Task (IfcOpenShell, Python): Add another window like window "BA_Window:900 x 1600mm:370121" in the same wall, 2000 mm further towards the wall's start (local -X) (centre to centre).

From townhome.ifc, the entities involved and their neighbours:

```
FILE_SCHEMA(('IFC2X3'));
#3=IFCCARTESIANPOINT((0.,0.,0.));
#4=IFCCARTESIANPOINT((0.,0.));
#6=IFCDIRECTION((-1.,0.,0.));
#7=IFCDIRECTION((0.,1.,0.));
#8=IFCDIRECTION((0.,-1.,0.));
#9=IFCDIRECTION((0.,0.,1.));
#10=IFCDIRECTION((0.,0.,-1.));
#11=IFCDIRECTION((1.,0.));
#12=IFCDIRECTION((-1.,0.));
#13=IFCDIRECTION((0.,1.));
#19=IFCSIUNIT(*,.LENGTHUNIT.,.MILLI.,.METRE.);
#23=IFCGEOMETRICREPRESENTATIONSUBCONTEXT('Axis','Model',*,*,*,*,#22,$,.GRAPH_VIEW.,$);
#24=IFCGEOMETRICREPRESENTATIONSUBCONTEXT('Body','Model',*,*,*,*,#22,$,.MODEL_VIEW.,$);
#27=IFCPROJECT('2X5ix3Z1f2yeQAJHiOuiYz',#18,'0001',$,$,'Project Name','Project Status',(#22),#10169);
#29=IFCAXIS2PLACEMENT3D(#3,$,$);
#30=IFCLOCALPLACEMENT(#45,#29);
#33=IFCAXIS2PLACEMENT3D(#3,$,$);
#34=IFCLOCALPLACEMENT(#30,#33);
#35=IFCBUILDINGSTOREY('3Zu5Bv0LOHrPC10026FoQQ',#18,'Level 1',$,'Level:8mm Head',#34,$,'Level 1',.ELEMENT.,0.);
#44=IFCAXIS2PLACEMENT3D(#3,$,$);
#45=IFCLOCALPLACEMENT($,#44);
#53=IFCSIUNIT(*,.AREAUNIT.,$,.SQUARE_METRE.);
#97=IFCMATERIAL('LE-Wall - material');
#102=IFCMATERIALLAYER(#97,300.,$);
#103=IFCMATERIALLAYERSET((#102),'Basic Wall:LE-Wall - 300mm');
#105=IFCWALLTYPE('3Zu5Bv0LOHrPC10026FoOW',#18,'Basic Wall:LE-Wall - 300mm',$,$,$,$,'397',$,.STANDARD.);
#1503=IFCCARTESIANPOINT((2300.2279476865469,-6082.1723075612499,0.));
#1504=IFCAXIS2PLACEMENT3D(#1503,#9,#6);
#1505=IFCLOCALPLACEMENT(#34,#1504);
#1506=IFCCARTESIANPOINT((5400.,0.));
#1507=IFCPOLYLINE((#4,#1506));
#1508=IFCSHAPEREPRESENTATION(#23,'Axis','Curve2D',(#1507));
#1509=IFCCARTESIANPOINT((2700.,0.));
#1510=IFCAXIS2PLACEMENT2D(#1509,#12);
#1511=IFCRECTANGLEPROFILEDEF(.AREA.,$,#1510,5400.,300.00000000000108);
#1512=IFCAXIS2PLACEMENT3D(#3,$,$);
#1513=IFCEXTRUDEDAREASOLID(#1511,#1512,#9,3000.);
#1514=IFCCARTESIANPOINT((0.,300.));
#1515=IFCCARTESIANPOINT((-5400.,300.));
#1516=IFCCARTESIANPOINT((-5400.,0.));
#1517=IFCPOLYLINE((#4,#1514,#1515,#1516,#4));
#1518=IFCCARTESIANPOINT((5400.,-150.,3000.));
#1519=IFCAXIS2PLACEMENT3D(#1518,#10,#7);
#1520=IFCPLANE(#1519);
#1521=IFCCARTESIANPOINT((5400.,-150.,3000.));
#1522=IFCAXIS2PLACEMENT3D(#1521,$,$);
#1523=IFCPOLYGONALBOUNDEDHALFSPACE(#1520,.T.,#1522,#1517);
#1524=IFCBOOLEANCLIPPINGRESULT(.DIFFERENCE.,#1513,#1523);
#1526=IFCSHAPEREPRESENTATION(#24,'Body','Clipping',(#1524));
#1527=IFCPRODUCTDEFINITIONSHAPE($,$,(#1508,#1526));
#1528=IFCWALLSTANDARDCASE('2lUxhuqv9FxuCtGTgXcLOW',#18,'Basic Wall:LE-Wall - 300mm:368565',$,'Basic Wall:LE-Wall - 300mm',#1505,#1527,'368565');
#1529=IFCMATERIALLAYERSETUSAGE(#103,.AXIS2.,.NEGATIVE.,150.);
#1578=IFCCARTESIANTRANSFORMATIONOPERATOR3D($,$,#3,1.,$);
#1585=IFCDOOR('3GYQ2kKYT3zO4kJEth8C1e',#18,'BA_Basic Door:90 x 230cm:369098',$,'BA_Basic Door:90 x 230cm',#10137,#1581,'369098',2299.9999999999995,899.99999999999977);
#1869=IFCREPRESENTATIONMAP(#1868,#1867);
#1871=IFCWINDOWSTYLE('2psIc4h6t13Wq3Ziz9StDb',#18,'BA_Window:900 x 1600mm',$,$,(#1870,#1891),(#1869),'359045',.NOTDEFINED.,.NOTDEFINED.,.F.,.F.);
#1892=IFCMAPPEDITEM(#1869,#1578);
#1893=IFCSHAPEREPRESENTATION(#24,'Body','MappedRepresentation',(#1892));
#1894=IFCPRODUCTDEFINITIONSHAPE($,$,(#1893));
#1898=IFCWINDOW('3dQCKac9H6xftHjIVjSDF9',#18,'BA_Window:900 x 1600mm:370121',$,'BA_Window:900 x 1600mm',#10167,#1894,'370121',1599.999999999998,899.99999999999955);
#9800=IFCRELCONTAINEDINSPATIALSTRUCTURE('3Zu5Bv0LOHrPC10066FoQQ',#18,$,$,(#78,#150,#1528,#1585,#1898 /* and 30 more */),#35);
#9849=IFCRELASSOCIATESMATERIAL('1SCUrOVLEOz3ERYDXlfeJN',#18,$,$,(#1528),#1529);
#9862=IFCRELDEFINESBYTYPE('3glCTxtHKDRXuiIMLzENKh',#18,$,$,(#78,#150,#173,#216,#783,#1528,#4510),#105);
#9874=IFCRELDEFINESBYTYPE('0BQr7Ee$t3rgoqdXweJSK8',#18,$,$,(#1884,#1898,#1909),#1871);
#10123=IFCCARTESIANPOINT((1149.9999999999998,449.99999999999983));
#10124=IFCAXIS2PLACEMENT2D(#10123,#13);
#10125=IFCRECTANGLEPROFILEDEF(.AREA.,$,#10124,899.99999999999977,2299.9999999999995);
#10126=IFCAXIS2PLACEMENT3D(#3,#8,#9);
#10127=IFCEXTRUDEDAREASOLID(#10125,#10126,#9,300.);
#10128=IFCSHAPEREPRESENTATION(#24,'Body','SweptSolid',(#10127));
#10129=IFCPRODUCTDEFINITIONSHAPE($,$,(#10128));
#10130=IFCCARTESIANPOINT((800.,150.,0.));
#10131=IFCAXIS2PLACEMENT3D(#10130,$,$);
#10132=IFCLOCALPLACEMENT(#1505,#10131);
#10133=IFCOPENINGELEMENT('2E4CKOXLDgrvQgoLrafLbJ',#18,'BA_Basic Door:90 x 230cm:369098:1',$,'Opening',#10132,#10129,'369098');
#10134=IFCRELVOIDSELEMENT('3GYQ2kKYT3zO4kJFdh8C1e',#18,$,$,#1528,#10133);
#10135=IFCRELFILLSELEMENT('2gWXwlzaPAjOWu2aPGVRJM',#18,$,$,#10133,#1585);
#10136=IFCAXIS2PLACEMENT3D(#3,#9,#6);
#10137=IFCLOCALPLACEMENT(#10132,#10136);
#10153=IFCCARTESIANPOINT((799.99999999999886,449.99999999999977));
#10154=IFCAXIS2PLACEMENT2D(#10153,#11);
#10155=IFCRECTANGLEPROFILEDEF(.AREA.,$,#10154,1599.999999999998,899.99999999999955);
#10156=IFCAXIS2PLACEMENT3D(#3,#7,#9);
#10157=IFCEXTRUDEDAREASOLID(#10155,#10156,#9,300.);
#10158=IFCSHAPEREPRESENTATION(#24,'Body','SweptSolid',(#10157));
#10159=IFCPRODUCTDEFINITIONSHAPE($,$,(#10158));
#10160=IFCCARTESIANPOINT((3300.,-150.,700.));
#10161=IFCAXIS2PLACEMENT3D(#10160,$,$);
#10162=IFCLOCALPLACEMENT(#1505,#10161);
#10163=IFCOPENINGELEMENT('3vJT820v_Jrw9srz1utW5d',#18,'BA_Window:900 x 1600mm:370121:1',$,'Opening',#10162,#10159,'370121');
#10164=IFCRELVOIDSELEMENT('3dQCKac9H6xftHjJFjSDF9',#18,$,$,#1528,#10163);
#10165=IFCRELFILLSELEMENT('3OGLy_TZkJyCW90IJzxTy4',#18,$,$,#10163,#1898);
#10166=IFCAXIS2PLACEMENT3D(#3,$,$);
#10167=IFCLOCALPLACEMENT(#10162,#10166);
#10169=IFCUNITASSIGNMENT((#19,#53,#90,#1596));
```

```python
import ifcopenshell
import ifcopenshell.api.feature
import ifcopenshell.api.geometry
import ifcopenshell.api.root
import ifcopenshell.geom
import ifcopenshell.util.element
import ifcopenshell.util.placement
import ifcopenshell.util.shape
import ifcopenshell.util.unit

model = ifcopenshell.open("townhome.ifc")
unit_scale = ifcopenshell.util.unit.calculate_unit_scale(model)
settings = ifcopenshell.geom.settings()


def volume(element):
    """Net volume in cubic metres, openings subtracted."""
    shape = ifcopenshell.geom.create_shape(settings, element)
    return ifcopenshell.util.shape.get_volume(shape.geometry)


def reuse_history(source, copy):
    """copy_class also copies each property set's owner history, people and application; keep the originals."""
    for rel in copy.IsDefinedBy:
        if rel.is_a("IfcRelDefinesByProperties") and (history := rel.RelatingPropertyDefinition.OwnerHistory):
            rel.RelatingPropertyDefinition.OwnerHistory = source.OwnerHistory
            ifcopenshell.util.element.remove_deep2(model, history)


window = model.by_guid("3dQCKac9H6xftHjIVjSDF9")
opening = window.FillsVoids[0].RelatingOpeningElement
wall = opening.VoidsElements[0].RelatingBuildingElement
before = volume(wall)
shift = ifcopenshell.util.placement.get_local_placement(wall.ObjectPlacement)[:3, 0] * -2 / unit_scale

# copy_class copies the void relationship, type, container and properties, but no geometry.
new_opening = ifcopenshell.api.root.copy_class(model, product=opening)
new_opening.Representation = ifcopenshell.util.element.copy_deep(
    model, opening.Representation, exclude=["IfcGeometricRepresentationContext", "IfcRepresentationMap"]
)
new_opening.Name = "BA_Window:900 x 1600mm"
new_opening.Tag = None
new_window = ifcopenshell.api.root.copy_class(model, product=window)
new_window.Representation = ifcopenshell.util.element.copy_deep(
    model, window.Representation, exclude=["IfcGeometricRepresentationContext", "IfcRepresentationMap"]
)
new_window.Name = "BA_Window:900 x 1600mm"
new_window.Tag = None
reuse_history(window, new_window)
fills = ifcopenshell.api.feature.add_filling(model, opening=new_opening, element=new_window)
fills.OwnerHistory = new_window.OwnerHistory  # required in IFC2X3

for old, new in ((opening, new_opening), (window, new_window)):
    matrix = ifcopenshell.util.placement.get_local_placement(old.ObjectPlacement)
    matrix[:3, 3] += shift
    ifcopenshell.api.geometry.edit_object_placement(model, product=new, matrix=matrix, is_si=False)

after = volume(wall)

print(f"wall volume {before:.3f} -> {after:.3f} m3")

model.write("townhome-out.ifc")
```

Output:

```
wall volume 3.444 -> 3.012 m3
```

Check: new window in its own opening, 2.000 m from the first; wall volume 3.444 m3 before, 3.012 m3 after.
